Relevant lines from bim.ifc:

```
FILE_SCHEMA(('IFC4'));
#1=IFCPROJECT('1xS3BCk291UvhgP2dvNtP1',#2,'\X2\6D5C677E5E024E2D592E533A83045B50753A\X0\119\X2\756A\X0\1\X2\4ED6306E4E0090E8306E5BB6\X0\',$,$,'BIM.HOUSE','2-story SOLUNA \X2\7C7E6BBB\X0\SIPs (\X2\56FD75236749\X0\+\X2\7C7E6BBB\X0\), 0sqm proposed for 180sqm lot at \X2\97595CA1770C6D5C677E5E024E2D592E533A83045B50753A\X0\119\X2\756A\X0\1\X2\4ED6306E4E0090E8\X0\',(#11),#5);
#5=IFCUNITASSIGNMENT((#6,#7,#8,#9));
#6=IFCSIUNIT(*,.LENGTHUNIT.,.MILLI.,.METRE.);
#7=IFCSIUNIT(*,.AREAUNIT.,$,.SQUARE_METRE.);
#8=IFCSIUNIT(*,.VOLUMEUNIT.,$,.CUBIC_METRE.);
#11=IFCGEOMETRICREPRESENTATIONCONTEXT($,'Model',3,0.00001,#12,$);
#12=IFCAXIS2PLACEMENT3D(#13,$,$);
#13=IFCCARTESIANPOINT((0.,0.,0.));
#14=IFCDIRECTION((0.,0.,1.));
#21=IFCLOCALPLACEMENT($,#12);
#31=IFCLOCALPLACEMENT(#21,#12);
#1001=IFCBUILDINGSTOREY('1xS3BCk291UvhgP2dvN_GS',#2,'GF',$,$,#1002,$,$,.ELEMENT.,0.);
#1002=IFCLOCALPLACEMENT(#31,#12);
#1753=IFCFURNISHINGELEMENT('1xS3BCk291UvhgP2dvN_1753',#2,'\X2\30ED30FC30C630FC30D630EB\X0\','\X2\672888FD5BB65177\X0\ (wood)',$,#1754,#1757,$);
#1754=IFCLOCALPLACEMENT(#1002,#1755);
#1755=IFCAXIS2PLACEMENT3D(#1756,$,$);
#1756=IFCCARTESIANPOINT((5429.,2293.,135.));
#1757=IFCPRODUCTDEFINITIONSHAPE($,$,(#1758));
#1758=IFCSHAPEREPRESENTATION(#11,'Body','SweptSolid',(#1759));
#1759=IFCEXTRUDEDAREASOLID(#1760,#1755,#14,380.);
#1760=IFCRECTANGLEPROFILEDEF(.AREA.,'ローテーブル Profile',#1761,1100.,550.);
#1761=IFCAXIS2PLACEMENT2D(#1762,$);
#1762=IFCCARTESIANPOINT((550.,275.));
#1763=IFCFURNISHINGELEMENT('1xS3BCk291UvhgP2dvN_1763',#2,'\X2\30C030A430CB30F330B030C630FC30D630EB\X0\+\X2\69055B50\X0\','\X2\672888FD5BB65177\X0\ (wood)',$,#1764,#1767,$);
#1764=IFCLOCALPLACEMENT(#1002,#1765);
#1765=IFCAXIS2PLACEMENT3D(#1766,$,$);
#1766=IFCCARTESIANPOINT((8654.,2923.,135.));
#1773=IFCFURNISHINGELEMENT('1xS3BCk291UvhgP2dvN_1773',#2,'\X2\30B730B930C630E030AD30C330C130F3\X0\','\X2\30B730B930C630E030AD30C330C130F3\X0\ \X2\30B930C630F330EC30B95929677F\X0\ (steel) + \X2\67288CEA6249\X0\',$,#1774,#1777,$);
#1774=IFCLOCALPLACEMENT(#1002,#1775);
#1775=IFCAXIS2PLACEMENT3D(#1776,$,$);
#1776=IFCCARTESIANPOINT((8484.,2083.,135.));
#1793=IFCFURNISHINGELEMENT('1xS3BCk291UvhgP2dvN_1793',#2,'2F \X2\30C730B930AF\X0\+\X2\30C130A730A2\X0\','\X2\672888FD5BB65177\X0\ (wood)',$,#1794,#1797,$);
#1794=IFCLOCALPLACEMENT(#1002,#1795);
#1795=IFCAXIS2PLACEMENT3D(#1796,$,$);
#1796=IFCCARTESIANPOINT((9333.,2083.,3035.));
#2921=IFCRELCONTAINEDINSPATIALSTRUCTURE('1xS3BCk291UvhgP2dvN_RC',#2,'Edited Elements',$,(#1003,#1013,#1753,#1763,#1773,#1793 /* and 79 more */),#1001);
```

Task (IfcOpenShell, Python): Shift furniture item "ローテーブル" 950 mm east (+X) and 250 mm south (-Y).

```python
import ifcopenshell
import ifcopenshell.api.geometry
import ifcopenshell.util.placement

model = ifcopenshell.open("bim.ifc")

item = model.by_guid("1xS3BCk291UvhgP2dvN_1753")
matrix = ifcopenshell.util.placement.get_local_placement(item.ObjectPlacement)
matrix[0, 3] += 950.0
matrix[1, 3] -= 250.0
ifcopenshell.api.geometry.edit_object_placement(model, product=item, matrix=matrix, is_si=False)

print(ifcopenshell.util.placement.get_local_placement(item.ObjectPlacement).round(3) + 0.0)

model.write("bim_v2.ifc")
```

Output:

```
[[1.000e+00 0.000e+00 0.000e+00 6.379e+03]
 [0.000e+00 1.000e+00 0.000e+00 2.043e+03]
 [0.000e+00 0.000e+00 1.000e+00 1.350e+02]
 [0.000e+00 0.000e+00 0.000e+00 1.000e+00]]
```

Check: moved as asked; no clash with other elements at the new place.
